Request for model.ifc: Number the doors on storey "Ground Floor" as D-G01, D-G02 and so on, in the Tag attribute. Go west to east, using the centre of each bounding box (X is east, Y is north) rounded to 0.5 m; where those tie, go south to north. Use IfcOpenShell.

First a look at what the model holds.

```python
import ifcopenshell
import ifcopenshell.util.element
import ifcopenshell.util.placement

model = ifcopenshell.open("model.ifc")
print(model.schema)
storey = next(s for s in model.by_type("IfcBuildingStorey") if s.Name == "Ground Floor")
doors = [e for e in ifcopenshell.util.element.get_decomposition(storey) if e.is_a("IfcDoor")]
for e in sorted(doors, key=lambda e: e.id()):
    origin = ifcopenshell.util.placement.get_local_placement(e.ObjectPlacement)[:3, 3]
    print(e.id(), e.Tag, e.Name, origin.round(2) + 0.0, sep=" | ")
```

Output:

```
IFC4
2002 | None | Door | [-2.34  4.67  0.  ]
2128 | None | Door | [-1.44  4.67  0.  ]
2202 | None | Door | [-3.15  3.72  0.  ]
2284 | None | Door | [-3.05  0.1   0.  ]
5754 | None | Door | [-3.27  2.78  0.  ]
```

```python
import ifcopenshell
import ifcopenshell.geom
import ifcopenshell.util.element
import ifcopenshell.util.shape

model = ifcopenshell.open("model.ifc")
settings = ifcopenshell.geom.settings()
settings.set("use-world-coords", True)


def centre(element):
    shape = ifcopenshell.geom.create_shape(settings, element)
    return ifcopenshell.util.shape.get_bbox_centroid(shape.geometry)


storey = next(s for s in model.by_type("IfcBuildingStorey") if s.Name == "Ground Floor")
doors = [e for e in ifcopenshell.util.element.get_decomposition(storey) if e.is_a("IfcDoor")]

# Insertion points can sit at a corner or the storey origin, so sort by the geometry (in metres).
centres = {e: centre(e) for e in doors}
doors.sort(key=lambda e: (round(centres[e][0] / 0.5), centres[e][1]))

for i, e in enumerate(doors, start=1):
    number = f"D-G{i:02d}"
    e.Tag = number
    print(e.id(), number)

model.write("model-out.ifc")
```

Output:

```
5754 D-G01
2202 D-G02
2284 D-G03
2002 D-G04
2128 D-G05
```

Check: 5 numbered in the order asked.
